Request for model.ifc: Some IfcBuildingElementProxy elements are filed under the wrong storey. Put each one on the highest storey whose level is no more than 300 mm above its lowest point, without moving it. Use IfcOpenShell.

First a look at what the model holds.

```python
import ifcopenshell
import ifcopenshell.util.element
import ifcopenshell.util.placement

model = ifcopenshell.open("model.ifc")
print(model.schema)
for storey in model.by_type("IfcBuildingStorey"):
    level = ifcopenshell.util.placement.get_storey_elevation(storey)
    count = sum(e.is_a("IfcBuildingElementProxy") for e in ifcopenshell.util.element.get_contained(storey))
    print(storey.id(), storey.Name, round(level, 3), count, sep=" | ")
```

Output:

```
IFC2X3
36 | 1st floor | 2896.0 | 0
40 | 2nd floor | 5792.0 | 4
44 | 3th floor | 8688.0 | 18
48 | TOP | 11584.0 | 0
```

```python
import ifcopenshell
import ifcopenshell.api.spatial
import ifcopenshell.geom
import ifcopenshell.util.element
import ifcopenshell.util.placement
import ifcopenshell.util.shape
import ifcopenshell.util.unit

model = ifcopenshell.open("model.ifc")
unit_scale = ifcopenshell.util.unit.calculate_unit_scale(model)
settings = ifcopenshell.geom.settings()

levels = sorted(
    ((ifcopenshell.util.placement.get_storey_elevation(s) * unit_scale, s) for s in model.by_type("IfcBuildingStorey")),
    key=lambda pair: pair[0],
)

for e in model.by_type("IfcBuildingElementProxy"):
    current = e.ContainedInStructure[0].RelatingStructure if e.ContainedInStructure else None
    if current is None or not current.is_a("IfcBuildingStorey"):
        continue
    shape = ifcopenshell.geom.create_shape(settings, e)
    bottom = ifcopenshell.util.shape.get_shape_bottom_elevation(shape, shape.geometry)
    below = [s for level, s in levels if level <= bottom + 0.3]
    storey = below[-1] if below else levels[0][1]
    if storey != current:
        # assign_container keeps the world position.
        ifcopenshell.api.spatial.assign_container(model, products=[e], relating_structure=storey)
        print(e.id(), current.Name, "->", storey.Name)

model.write("model_v2.ifc")
```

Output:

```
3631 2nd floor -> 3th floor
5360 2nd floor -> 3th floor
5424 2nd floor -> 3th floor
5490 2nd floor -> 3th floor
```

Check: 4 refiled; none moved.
